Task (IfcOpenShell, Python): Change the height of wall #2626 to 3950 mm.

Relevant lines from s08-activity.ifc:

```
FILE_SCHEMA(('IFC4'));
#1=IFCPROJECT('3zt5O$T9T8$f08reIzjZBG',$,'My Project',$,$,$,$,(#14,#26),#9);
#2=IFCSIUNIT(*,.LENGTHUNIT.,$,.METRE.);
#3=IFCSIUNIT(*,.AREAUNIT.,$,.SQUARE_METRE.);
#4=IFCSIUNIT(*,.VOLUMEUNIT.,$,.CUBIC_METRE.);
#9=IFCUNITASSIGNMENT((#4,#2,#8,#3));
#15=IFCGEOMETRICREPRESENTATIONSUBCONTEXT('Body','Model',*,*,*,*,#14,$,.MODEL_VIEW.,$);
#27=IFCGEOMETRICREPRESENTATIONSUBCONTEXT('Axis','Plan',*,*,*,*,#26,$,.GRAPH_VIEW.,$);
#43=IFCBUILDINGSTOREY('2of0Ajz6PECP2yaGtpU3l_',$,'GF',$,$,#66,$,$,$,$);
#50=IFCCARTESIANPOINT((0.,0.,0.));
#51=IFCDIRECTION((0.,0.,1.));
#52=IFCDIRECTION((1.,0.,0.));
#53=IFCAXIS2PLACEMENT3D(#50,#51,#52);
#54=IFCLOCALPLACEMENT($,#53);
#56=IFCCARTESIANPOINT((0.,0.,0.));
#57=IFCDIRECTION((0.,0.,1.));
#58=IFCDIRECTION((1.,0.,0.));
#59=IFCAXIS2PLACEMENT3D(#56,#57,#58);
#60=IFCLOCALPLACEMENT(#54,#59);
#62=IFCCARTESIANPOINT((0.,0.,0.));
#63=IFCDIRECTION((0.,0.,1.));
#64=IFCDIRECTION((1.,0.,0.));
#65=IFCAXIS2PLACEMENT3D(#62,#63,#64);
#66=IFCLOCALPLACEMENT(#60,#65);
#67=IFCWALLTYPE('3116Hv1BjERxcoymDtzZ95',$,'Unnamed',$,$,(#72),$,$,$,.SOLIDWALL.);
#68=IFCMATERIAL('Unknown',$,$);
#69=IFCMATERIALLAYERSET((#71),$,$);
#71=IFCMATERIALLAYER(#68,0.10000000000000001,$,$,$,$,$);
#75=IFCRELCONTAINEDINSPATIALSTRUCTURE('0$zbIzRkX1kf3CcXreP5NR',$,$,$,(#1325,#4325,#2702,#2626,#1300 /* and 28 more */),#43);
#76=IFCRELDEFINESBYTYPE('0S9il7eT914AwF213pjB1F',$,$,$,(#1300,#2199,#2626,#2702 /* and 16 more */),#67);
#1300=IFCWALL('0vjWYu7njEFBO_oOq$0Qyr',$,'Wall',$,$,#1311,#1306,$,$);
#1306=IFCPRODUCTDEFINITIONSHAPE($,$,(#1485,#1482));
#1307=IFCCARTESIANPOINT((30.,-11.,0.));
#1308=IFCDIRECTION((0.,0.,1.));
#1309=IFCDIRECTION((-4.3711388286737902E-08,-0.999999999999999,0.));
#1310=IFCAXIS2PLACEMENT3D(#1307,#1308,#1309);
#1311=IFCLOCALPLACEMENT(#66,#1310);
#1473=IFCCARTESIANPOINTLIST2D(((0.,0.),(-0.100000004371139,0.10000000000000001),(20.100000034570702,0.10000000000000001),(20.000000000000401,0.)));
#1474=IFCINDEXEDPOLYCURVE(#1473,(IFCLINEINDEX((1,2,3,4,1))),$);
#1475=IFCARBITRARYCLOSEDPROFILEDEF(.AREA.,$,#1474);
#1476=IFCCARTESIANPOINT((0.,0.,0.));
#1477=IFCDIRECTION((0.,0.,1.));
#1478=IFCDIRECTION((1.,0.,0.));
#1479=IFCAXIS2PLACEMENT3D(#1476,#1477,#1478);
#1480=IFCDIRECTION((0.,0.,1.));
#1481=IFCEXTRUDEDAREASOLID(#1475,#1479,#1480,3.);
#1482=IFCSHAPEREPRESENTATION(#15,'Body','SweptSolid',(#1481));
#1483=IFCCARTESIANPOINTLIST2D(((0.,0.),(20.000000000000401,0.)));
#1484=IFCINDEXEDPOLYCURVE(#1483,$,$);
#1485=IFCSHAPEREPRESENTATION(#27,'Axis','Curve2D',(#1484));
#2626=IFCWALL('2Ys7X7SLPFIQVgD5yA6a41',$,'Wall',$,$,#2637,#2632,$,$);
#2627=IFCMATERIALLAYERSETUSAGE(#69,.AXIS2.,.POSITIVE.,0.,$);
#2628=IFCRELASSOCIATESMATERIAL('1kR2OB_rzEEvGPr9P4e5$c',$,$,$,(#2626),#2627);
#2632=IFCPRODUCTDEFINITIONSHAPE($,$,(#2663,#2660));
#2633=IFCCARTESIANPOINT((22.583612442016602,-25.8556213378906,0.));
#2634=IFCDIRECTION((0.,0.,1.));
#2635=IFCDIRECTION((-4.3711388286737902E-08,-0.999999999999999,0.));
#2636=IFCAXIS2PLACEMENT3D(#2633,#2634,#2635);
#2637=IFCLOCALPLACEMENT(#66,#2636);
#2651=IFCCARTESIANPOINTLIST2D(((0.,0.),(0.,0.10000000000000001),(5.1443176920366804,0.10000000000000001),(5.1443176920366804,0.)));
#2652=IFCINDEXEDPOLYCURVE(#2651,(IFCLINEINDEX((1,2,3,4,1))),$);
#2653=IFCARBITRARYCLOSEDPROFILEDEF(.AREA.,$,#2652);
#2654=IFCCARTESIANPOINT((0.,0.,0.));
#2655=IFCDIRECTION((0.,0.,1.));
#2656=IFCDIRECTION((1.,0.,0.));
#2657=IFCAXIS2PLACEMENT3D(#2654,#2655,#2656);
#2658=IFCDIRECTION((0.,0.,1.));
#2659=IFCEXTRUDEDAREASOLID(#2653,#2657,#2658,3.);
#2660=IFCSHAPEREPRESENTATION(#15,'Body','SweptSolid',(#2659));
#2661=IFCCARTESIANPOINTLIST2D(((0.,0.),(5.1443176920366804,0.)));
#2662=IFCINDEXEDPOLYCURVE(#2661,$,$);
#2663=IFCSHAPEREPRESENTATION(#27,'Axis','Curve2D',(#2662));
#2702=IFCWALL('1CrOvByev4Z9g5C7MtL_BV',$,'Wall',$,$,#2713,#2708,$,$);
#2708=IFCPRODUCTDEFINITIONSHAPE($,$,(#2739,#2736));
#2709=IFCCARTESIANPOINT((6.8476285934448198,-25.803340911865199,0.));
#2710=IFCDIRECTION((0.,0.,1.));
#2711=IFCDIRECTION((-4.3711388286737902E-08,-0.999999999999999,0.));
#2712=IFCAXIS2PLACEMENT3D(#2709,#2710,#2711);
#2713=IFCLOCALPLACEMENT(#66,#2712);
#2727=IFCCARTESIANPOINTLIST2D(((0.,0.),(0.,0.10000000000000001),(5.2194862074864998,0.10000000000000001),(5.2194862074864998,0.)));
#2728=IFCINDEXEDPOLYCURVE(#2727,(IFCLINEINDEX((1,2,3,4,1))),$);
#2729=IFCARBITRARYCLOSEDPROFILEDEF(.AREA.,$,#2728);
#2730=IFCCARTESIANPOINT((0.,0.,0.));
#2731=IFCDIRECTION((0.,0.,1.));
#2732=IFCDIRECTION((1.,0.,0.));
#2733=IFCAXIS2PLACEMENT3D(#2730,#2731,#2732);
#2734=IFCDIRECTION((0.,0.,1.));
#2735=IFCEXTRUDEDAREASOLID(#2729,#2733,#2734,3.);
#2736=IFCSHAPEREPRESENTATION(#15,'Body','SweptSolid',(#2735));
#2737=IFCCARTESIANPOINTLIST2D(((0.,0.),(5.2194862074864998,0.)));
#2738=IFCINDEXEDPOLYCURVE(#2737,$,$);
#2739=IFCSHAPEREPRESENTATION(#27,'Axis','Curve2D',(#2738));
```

```python
import ifcopenshell
import ifcopenshell.geom
import ifcopenshell.util.representation
import ifcopenshell.util.shape
import ifcopenshell.util.unit

model = ifcopenshell.open("s08-activity.ifc")
unit_scale = ifcopenshell.util.unit.calculate_unit_scale(model)
settings = ifcopenshell.geom.settings()


def volume(element):
    """Net volume in cubic metres, openings subtracted."""
    shape = ifcopenshell.geom.create_shape(settings, element)
    return ifcopenshell.util.shape.get_volume(shape.geometry)


wall = model.by_guid("2Ys7X7SLPFIQVgD5yA6a41")
before = volume(wall)

body = ifcopenshell.util.representation.get_representation(wall, "Model", "Body")
solid = body.Items[0]
old_height = solid.Depth
solid.Depth = 3.95 / unit_scale
after = volume(wall)

print(f"height {old_height:g} -> {solid.Depth:g}, volume {before:.3f} -> {after:.3f} m3")

model.write("s08-activity-out.ifc")
```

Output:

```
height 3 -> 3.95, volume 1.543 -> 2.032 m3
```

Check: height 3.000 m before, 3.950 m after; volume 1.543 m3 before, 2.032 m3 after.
